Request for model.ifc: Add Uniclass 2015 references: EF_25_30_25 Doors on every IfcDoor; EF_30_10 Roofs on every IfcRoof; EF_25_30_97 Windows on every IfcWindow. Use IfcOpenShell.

First a look at what the model holds.

```python
import ifcopenshell

model = ifcopenshell.open("model.ifc")
print(model.schema)
print("classifications:", [c.Name for c in model.by_type("IfcClassification")])
for ifc_class in ("IfcDoor", "IfcRoof", "IfcStair", "IfcWall", "IfcWindow"):
    print(ifc_class, len(model.by_type(ifc_class)))
```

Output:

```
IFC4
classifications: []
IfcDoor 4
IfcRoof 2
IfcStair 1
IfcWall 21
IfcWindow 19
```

```python
import ifcopenshell
import ifcopenshell.api.classification

model = ifcopenshell.open("model.ifc")

system = ifcopenshell.api.classification.add_classification(model, classification="Uniclass 2015")

codes = {
    "IfcDoor": ("EF_25_30_25", "Doors"),
    "IfcRoof": ("EF_30_10", "Roofs"),
    "IfcWindow": ("EF_25_30_97", "Windows"),
}
for ifc_class, (code, name) in codes.items():
    products = model.by_type(ifc_class)
    ifcopenshell.api.classification.add_reference(
        model, products=products, classification=system, identification=code, name=name
    )
    print(code, len(products))

model.write("model_updated.ifc")
```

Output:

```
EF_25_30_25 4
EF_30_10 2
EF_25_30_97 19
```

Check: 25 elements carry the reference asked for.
